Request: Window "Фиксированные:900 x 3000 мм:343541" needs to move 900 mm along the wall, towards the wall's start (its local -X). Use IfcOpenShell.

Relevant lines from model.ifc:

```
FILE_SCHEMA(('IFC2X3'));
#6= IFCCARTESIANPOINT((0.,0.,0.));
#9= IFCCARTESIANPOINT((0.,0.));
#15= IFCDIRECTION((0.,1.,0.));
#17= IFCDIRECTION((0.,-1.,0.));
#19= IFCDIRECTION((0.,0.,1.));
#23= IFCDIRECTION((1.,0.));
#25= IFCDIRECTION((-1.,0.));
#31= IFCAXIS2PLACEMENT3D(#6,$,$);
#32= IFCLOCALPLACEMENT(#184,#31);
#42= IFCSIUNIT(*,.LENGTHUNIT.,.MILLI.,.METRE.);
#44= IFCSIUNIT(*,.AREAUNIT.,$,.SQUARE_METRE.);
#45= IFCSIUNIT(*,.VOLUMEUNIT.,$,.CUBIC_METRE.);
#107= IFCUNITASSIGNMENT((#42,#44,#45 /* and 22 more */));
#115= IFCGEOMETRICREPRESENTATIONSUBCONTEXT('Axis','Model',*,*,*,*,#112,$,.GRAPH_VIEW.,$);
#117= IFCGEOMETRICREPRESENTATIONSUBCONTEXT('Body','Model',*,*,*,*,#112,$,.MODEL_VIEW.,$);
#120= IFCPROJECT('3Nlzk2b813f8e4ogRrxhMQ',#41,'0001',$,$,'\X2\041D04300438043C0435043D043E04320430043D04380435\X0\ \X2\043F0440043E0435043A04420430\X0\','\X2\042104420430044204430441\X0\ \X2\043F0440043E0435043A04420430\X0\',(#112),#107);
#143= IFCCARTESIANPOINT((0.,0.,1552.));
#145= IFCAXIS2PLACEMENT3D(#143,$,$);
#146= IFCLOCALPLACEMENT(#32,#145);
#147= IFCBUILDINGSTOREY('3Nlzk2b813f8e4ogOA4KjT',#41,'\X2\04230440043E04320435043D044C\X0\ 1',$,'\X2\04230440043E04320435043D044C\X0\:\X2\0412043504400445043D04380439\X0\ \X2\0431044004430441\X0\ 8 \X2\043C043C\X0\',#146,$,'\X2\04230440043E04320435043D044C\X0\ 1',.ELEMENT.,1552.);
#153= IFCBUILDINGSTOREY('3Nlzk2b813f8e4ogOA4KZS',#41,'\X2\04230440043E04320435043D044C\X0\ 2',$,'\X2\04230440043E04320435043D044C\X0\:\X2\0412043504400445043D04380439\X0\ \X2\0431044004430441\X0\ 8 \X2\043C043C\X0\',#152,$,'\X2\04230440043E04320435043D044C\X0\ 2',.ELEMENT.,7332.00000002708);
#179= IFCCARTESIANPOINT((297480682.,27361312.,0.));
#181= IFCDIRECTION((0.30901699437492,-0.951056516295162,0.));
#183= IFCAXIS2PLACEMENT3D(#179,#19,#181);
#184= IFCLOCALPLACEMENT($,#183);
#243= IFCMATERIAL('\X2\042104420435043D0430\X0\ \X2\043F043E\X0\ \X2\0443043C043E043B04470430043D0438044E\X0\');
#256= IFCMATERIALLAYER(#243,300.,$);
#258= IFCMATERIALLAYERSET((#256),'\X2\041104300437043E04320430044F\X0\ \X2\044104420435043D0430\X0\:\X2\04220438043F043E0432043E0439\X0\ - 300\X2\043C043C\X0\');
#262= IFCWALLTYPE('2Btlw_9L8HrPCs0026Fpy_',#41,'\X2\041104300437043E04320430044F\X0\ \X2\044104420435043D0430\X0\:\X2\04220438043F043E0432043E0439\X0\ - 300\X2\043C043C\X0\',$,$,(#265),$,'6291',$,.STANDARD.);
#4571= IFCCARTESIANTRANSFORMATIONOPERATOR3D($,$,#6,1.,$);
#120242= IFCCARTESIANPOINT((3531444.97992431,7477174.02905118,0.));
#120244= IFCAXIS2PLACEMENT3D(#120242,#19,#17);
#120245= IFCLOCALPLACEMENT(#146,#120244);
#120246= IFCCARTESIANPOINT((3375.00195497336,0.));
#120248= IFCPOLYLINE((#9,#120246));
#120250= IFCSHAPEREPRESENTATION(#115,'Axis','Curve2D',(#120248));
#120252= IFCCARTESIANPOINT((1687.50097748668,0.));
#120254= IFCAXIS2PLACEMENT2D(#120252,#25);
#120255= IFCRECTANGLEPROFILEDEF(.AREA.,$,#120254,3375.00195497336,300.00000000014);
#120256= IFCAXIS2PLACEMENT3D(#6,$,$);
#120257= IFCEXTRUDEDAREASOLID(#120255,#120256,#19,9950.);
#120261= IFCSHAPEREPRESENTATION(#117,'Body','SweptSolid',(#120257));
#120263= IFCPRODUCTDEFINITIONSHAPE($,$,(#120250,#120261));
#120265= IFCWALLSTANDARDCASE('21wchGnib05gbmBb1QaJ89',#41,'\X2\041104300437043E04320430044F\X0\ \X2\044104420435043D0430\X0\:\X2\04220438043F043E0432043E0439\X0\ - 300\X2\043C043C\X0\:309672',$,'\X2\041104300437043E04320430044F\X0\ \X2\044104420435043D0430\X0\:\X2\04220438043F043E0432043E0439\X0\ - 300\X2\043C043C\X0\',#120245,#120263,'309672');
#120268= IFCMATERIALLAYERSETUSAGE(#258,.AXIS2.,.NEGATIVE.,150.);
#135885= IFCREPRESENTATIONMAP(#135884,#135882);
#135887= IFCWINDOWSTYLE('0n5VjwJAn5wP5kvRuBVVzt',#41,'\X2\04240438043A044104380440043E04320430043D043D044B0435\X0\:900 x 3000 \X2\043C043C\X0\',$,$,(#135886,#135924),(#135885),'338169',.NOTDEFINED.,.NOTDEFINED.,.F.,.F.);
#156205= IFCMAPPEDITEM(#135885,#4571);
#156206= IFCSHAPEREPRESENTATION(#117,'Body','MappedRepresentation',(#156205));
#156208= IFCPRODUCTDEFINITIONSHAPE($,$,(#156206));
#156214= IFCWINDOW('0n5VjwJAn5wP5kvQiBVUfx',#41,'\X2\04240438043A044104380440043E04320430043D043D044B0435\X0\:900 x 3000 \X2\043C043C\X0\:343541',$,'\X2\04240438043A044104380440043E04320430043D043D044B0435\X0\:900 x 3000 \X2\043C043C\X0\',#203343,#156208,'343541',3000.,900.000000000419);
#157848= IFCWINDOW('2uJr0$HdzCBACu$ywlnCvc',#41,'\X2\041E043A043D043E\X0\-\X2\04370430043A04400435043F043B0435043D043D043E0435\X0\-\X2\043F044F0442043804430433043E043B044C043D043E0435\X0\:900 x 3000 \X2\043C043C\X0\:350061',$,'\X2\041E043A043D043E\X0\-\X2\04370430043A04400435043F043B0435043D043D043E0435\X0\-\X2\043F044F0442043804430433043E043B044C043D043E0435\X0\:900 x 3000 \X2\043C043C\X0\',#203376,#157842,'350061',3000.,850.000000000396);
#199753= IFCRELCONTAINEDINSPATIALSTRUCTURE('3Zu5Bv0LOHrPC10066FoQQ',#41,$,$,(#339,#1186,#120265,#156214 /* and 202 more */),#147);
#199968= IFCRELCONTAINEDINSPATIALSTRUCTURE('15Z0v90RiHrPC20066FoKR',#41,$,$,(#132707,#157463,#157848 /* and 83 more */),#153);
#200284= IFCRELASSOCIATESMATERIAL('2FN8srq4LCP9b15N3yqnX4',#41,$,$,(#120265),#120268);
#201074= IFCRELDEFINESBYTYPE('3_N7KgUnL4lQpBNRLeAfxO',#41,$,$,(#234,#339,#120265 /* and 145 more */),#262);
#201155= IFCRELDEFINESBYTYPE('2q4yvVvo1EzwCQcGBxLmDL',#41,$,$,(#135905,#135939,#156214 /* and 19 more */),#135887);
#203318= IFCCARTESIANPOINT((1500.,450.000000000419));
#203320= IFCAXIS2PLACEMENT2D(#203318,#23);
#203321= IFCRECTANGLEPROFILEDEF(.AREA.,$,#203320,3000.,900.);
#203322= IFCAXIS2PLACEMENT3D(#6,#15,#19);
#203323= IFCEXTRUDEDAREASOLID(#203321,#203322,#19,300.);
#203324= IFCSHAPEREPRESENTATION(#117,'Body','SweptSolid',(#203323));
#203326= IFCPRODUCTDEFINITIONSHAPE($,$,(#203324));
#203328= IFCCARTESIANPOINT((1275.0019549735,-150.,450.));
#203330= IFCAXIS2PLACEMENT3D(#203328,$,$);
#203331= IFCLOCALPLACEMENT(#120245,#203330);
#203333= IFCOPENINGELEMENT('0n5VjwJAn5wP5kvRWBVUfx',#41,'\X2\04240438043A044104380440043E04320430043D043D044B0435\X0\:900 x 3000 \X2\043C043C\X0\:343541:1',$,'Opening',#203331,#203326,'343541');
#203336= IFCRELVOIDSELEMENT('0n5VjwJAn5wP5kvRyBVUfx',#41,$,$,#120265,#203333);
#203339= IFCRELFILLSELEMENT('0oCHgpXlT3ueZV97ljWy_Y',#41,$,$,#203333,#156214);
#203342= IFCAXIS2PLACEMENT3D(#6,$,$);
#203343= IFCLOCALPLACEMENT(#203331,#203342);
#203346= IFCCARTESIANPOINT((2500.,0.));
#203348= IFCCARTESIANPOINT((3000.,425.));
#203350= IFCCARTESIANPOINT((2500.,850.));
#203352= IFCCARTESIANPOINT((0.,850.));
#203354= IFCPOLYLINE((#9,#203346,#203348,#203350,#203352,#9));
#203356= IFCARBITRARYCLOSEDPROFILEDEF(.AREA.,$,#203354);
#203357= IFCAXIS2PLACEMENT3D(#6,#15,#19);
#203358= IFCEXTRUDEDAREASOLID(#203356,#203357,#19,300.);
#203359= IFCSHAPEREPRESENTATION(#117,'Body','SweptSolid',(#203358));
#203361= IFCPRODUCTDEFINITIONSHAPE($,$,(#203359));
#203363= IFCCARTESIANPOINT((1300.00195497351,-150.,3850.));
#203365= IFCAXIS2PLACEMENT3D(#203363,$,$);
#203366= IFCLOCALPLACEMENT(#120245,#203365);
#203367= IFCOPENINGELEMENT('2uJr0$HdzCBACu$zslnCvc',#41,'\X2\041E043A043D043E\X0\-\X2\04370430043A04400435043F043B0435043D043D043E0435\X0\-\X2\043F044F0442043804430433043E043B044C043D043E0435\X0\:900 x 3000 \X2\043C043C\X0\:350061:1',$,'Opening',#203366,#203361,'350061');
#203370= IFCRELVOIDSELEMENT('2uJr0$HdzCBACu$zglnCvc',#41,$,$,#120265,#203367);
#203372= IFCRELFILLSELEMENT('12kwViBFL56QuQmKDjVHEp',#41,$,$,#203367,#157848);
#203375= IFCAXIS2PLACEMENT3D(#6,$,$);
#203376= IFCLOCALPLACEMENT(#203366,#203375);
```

```python
import ifcopenshell
import ifcopenshell.api.geometry
import ifcopenshell.util.placement

model = ifcopenshell.open("model.ifc")

window = model.by_id(156214)
opening = window.FillsVoids[0].RelatingOpeningElement
wall = opening.VoidsElements[0].RelatingBuildingElement

wall_matrix = ifcopenshell.util.placement.get_local_placement(wall.ObjectPlacement)
shift = wall_matrix[:3, 0] * -900.0
before = ifcopenshell.util.placement.get_local_placement(window.ObjectPlacement)[:3, 3].copy()

# The window is placed relative to its opening, so it follows when the opening moves.
matrix = ifcopenshell.util.placement.get_local_placement(opening.ObjectPlacement)
matrix[:3, 3] += shift
ifcopenshell.api.geometry.edit_object_placement(
    model, product=opening, matrix=matrix, is_si=False, should_transform_children=True
)

after = ifcopenshell.util.placement.get_local_placement(window.ObjectPlacement)[:3, 3]
print("window moved by", (after - before).round(3) + 0.0)

model.write("model-out.ifc")
```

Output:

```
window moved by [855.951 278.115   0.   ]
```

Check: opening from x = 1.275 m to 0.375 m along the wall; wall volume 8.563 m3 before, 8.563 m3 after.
